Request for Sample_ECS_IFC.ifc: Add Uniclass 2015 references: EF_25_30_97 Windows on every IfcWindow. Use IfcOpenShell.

First a look at what the model holds.

```python
import ifcopenshell

model = ifcopenshell.open("Sample_ECS_IFC.ifc")
print(model.schema)
print("classifications:", [c.Name for c in model.by_type("IfcClassification")])
for ifc_class in ("IfcDoor", "IfcRoof", "IfcStair", "IfcWall", "IfcWindow"):
    print(ifc_class, len(model.by_type(ifc_class)))
```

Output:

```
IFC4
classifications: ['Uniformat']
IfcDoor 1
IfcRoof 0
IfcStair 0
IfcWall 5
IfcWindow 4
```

```python
import ifcopenshell
import ifcopenshell.api.classification

model = ifcopenshell.open("Sample_ECS_IFC.ifc")

system = ifcopenshell.api.classification.add_classification(model, classification="Uniclass 2015")

codes = {
    "IfcWindow": ("EF_25_30_97", "Windows"),
}
for ifc_class, (code, name) in codes.items():
    products = model.by_type(ifc_class)
    ifcopenshell.api.classification.add_reference(
        model, products=products, classification=system, identification=code, name=name
    )
    print(code, len(products))

model.write("Sample_ECS_IFC_updated.ifc")
```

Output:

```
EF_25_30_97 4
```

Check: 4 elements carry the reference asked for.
